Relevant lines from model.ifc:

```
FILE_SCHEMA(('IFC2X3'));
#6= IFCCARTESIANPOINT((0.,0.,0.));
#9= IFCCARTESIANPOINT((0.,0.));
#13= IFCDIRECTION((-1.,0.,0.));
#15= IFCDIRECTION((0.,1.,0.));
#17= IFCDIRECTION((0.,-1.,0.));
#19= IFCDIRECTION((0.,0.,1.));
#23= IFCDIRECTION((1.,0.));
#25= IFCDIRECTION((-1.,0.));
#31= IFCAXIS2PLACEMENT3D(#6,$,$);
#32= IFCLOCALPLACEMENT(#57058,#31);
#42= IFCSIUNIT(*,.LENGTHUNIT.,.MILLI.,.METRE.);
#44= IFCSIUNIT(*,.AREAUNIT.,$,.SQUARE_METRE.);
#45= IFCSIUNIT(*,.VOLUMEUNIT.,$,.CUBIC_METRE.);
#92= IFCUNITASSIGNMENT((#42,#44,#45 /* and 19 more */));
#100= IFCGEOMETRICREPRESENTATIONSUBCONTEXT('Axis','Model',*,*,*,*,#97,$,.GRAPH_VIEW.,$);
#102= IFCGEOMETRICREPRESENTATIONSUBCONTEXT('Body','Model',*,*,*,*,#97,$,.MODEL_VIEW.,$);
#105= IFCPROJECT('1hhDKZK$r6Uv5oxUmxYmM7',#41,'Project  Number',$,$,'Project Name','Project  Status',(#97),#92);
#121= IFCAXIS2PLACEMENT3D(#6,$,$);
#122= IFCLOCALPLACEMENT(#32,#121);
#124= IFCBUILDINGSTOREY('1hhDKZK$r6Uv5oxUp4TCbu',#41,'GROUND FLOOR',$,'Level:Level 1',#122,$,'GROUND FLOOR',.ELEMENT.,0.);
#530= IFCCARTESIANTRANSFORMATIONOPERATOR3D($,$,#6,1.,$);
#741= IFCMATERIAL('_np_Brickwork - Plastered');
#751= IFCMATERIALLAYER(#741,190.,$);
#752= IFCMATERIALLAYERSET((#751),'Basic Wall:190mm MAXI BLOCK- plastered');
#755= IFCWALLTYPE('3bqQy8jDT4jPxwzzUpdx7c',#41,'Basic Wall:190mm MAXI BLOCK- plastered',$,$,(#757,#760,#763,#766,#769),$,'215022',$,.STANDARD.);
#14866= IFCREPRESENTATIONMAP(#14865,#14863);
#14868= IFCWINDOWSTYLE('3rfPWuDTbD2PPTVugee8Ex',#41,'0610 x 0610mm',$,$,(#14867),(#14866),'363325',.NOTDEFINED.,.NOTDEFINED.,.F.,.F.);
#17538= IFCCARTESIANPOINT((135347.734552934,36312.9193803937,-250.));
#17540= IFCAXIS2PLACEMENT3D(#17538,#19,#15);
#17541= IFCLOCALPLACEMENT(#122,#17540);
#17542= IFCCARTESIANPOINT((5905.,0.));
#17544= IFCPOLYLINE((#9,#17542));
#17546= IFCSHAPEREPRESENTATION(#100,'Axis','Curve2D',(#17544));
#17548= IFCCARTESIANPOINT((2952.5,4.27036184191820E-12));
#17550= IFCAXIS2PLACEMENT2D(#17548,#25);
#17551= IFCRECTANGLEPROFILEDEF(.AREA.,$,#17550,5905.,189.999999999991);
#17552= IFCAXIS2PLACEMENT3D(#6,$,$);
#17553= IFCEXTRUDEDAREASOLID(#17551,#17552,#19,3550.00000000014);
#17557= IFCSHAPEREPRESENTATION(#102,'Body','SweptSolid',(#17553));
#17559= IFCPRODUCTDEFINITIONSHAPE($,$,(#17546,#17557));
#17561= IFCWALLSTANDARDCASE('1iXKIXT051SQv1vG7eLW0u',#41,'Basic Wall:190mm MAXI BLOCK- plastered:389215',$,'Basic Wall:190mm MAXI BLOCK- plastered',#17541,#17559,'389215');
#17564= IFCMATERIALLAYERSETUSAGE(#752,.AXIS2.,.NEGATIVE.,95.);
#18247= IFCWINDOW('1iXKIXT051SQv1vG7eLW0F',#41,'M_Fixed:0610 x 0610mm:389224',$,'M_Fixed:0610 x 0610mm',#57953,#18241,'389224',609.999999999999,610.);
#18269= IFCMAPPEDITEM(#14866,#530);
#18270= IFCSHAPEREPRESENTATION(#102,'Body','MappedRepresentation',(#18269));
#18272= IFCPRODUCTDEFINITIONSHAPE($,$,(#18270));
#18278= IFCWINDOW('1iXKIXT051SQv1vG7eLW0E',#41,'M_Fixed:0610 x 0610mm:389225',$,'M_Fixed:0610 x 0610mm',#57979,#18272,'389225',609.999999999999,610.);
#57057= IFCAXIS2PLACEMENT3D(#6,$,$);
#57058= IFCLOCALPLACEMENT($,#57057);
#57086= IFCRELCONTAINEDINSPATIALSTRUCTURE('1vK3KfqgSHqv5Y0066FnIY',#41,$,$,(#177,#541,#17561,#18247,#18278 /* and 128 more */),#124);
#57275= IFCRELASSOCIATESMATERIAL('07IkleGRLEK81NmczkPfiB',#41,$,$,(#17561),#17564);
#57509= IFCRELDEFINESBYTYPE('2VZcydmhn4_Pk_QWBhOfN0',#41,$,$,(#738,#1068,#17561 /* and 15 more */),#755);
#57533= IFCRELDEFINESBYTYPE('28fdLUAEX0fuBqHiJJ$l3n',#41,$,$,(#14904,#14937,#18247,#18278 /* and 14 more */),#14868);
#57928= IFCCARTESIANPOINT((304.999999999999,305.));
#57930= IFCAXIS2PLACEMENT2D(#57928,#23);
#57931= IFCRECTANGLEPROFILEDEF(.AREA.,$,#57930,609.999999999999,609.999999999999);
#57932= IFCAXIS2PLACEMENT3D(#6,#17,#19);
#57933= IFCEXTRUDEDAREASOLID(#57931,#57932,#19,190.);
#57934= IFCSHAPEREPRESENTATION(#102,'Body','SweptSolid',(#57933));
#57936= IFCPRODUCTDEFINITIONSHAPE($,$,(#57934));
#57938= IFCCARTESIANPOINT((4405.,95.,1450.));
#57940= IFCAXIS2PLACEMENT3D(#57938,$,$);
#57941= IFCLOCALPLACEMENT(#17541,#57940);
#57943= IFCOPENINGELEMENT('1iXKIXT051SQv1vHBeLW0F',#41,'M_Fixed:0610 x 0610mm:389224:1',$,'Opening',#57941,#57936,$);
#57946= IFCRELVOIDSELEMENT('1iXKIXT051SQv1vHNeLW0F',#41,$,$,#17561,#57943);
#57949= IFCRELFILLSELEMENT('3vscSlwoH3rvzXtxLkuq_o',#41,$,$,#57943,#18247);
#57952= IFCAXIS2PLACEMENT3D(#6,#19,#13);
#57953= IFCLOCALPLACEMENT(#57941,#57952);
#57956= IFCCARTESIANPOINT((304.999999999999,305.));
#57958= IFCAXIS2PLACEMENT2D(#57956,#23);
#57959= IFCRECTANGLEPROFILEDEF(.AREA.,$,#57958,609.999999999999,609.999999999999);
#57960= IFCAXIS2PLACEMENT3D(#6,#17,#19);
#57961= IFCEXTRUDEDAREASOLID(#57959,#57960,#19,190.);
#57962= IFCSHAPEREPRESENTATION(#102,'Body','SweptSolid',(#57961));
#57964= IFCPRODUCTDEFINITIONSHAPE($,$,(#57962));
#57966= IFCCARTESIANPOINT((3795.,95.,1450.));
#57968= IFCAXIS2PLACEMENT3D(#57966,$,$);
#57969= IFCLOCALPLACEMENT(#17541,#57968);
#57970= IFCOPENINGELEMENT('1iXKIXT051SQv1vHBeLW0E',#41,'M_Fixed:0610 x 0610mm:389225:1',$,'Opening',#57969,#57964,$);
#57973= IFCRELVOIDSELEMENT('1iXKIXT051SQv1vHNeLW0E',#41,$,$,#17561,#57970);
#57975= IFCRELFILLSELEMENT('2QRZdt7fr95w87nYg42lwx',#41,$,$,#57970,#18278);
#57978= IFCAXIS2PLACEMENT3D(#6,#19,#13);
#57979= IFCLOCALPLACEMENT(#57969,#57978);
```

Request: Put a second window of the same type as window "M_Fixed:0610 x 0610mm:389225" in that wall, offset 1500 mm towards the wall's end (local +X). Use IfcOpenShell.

```python
import ifcopenshell
import ifcopenshell.api.feature
import ifcopenshell.api.geometry
import ifcopenshell.api.root
import ifcopenshell.geom
import ifcopenshell.util.element
import ifcopenshell.util.placement
import ifcopenshell.util.shape

model = ifcopenshell.open("model.ifc")
settings = ifcopenshell.geom.settings()


def volume(element):
    """Net volume in cubic metres, openings subtracted."""
    shape = ifcopenshell.geom.create_shape(settings, element)
    return ifcopenshell.util.shape.get_volume(shape.geometry)


def reuse_history(source, copy):
    """copy_class also copies each property set's owner history, people and application; keep the originals."""
    for rel in copy.IsDefinedBy:
        if rel.is_a("IfcRelDefinesByProperties") and (history := rel.RelatingPropertyDefinition.OwnerHistory):
            rel.RelatingPropertyDefinition.OwnerHistory = source.OwnerHistory
            ifcopenshell.util.element.remove_deep2(model, history)


window = model.by_guid("1iXKIXT051SQv1vG7eLW0E")
opening = window.FillsVoids[0].RelatingOpeningElement
wall = opening.VoidsElements[0].RelatingBuildingElement
before = volume(wall)
shift = ifcopenshell.util.placement.get_local_placement(wall.ObjectPlacement)[:3, 0] * 1500.0

# copy_class copies the void relationship, type, container and properties, but no geometry.
new_opening = ifcopenshell.api.root.copy_class(model, product=opening)
new_opening.Representation = ifcopenshell.util.element.copy_deep(
    model, opening.Representation, exclude=["IfcGeometricRepresentationContext", "IfcRepresentationMap"]
)
new_opening.Name = "M_Fixed:0610 x 0610mm"
new_window = ifcopenshell.api.root.copy_class(model, product=window)
new_window.Representation = ifcopenshell.util.element.copy_deep(
    model, window.Representation, exclude=["IfcGeometricRepresentationContext", "IfcRepresentationMap"]
)
new_window.Name = "M_Fixed:0610 x 0610mm"
new_window.Tag = None
reuse_history(window, new_window)
fills = ifcopenshell.api.feature.add_filling(model, opening=new_opening, element=new_window)
fills.OwnerHistory = new_window.OwnerHistory  # required in IFC2X3

for old, new in ((opening, new_opening), (window, new_window)):
    matrix = ifcopenshell.util.placement.get_local_placement(old.ObjectPlacement)
    matrix[:3, 3] += shift
    ifcopenshell.api.geometry.edit_object_placement(model, product=new, matrix=matrix, is_si=False)

after = volume(wall)

print(f"wall volume {before:.3f} -> {after:.3f} m3")

model.write("model_updated.ifc")
```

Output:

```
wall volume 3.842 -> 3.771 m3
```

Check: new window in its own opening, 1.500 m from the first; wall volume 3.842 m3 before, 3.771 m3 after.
